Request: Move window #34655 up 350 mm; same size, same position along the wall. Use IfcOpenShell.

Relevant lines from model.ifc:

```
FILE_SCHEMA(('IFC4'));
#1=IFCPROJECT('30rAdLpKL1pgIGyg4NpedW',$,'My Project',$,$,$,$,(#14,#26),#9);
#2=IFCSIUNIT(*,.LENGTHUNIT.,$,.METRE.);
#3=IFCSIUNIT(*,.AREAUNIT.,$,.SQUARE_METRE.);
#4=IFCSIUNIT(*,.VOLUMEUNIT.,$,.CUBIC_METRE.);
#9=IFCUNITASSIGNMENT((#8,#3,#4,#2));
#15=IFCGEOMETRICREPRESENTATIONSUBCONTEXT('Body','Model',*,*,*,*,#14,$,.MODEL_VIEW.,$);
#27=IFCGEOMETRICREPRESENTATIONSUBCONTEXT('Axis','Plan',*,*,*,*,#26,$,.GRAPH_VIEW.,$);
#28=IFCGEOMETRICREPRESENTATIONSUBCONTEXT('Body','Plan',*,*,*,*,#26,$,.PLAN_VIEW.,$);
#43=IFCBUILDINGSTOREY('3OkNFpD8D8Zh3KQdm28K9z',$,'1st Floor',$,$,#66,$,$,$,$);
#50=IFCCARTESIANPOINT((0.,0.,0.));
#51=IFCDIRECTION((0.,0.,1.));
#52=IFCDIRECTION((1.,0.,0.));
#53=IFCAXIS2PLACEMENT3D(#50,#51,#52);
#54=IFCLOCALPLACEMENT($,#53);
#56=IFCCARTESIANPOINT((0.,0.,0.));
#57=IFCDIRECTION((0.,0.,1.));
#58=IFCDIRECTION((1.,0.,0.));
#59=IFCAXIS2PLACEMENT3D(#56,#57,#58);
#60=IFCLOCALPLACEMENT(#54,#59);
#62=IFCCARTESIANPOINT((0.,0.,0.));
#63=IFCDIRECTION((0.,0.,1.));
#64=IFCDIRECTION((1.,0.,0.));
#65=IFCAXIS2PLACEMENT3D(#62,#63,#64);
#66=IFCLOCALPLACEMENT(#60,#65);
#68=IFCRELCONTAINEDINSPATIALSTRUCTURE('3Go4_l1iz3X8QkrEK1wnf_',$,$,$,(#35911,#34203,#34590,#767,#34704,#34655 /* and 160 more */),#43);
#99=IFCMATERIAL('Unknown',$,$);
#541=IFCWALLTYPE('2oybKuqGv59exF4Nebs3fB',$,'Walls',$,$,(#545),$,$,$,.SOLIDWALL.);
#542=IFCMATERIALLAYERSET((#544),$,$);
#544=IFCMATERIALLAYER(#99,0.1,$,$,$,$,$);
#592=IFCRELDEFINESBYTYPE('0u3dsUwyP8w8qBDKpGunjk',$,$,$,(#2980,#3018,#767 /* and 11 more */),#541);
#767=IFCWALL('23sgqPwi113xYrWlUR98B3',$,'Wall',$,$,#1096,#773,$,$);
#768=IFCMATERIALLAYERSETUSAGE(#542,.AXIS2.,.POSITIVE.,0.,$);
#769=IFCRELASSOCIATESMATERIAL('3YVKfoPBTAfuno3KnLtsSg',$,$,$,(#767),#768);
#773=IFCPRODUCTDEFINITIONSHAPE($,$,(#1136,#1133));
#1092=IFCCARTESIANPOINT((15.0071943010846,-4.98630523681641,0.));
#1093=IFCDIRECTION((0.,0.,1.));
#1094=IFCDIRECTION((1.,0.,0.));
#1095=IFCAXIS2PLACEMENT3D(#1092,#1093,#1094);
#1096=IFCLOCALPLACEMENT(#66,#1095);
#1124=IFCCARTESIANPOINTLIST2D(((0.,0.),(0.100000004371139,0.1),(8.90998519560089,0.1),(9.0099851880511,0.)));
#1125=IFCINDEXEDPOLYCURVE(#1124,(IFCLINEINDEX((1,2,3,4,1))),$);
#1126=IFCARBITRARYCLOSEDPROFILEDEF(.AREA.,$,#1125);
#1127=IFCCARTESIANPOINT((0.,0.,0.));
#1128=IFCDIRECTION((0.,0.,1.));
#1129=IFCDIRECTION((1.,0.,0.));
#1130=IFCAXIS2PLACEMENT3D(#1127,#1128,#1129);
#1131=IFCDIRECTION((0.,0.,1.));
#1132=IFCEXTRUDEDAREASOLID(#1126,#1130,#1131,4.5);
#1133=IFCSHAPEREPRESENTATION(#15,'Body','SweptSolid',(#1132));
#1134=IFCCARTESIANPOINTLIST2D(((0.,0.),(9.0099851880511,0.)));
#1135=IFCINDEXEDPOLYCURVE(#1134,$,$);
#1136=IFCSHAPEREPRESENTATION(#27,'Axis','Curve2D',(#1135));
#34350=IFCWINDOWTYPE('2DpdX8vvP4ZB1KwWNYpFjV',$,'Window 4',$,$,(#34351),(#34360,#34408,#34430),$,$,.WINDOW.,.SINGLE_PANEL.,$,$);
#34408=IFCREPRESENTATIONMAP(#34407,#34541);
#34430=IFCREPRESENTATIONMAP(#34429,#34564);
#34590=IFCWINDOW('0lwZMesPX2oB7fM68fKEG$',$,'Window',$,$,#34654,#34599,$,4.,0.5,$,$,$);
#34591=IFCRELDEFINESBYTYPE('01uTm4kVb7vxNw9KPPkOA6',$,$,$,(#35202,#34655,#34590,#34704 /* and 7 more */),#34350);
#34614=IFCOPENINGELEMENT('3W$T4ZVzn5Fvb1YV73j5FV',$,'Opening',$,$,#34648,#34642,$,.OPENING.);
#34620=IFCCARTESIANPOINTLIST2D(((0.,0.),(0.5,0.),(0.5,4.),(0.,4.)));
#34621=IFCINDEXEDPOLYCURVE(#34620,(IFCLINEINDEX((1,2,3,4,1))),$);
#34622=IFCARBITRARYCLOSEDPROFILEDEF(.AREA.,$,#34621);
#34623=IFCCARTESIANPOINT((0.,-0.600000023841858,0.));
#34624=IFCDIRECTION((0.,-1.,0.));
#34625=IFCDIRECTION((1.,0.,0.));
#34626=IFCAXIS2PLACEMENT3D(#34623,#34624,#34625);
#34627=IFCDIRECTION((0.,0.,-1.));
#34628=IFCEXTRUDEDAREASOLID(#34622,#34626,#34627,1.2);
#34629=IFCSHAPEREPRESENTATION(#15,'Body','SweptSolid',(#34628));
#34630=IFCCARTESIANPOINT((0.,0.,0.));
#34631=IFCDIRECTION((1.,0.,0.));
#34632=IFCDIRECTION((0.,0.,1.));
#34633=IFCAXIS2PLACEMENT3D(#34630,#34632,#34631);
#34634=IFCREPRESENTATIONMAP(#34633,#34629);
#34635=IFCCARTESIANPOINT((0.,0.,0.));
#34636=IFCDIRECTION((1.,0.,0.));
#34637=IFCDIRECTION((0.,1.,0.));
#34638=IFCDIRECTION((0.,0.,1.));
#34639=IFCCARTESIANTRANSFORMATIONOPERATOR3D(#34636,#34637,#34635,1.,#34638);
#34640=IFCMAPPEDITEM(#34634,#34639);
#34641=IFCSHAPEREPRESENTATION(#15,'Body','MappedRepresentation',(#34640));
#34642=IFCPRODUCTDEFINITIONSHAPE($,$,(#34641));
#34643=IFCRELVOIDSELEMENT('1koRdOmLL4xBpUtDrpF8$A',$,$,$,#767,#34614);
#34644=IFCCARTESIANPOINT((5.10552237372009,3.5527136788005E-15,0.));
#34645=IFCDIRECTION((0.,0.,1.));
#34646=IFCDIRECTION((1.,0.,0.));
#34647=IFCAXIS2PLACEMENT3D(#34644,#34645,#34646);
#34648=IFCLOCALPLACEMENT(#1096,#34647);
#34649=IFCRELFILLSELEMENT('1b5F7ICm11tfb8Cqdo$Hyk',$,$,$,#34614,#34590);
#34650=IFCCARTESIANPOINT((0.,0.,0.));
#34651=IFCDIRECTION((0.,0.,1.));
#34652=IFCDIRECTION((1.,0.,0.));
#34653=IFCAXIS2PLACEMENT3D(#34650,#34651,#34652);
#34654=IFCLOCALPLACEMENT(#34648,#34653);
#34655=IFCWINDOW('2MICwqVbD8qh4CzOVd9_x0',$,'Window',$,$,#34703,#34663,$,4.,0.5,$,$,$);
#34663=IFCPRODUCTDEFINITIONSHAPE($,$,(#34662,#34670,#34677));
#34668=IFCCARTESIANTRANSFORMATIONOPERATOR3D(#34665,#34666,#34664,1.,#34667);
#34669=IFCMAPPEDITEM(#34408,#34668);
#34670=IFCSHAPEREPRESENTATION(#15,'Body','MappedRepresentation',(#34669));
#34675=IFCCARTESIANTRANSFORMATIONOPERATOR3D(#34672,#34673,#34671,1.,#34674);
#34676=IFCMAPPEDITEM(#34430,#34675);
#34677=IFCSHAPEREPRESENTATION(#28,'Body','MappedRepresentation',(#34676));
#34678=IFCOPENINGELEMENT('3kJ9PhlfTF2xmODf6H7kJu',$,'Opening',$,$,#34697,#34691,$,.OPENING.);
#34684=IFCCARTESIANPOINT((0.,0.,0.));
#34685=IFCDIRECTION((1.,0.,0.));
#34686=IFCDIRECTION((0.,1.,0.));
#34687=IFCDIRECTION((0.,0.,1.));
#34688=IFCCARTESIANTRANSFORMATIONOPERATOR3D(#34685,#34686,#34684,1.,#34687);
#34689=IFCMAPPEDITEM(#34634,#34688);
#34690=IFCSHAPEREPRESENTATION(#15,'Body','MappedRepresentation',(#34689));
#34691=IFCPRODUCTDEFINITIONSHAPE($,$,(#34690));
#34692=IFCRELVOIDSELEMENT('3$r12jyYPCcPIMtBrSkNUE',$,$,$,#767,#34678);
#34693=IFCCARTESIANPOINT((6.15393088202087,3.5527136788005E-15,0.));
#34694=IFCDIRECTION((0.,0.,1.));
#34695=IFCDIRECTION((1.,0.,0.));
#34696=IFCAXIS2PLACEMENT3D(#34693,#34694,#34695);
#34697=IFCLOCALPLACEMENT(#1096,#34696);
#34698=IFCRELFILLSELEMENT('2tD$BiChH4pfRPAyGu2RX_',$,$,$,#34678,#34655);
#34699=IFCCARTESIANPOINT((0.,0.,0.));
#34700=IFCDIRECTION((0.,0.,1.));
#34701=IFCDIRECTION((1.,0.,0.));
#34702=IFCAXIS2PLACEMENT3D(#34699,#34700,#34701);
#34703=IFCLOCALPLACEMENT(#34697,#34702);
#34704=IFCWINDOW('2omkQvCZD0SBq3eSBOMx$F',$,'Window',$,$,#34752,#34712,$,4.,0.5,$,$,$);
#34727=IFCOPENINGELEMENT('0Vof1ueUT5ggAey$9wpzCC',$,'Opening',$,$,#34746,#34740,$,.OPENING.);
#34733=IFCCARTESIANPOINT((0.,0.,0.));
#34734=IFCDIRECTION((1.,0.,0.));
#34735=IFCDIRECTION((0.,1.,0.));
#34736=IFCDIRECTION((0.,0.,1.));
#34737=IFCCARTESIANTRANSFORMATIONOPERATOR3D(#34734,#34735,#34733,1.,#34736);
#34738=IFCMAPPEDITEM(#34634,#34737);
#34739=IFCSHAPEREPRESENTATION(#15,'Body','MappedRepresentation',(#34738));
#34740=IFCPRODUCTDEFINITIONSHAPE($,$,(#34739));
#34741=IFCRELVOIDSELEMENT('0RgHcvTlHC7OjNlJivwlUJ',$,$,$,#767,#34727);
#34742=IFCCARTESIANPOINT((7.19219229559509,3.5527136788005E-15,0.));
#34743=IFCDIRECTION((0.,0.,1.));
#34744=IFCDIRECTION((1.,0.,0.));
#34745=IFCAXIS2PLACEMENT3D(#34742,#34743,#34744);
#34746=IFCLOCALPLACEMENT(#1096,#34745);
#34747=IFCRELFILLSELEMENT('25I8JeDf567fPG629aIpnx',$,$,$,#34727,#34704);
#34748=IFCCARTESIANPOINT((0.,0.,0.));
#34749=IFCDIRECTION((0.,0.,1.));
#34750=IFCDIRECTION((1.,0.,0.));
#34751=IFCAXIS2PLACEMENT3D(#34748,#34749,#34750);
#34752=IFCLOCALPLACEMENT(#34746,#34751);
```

```python
import numpy as np
import ifcopenshell
import ifcopenshell.api.geometry
import ifcopenshell.util.placement
import ifcopenshell.util.unit

model = ifcopenshell.open("model.ifc")
unit_scale = ifcopenshell.util.unit.calculate_unit_scale(model)

window = model.by_guid("2MICwqVbD8qh4CzOVd9_x0")
opening = window.FillsVoids[0].RelatingOpeningElement
dz = 0.35 / unit_scale

shift = np.array([0.0, 0.0, dz])
# The window is placed relative to its opening, so it follows when the opening moves.
matrix = ifcopenshell.util.placement.get_local_placement(opening.ObjectPlacement)
matrix[:3, 3] += shift
ifcopenshell.api.geometry.edit_object_placement(
    model, product=opening, matrix=matrix, is_si=False, should_transform_children=True
)

print(f"moved by {dz * unit_scale:+.3f} m")

model.write("model_updated.ifc")
```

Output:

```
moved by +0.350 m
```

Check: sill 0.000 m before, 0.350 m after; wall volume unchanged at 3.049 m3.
